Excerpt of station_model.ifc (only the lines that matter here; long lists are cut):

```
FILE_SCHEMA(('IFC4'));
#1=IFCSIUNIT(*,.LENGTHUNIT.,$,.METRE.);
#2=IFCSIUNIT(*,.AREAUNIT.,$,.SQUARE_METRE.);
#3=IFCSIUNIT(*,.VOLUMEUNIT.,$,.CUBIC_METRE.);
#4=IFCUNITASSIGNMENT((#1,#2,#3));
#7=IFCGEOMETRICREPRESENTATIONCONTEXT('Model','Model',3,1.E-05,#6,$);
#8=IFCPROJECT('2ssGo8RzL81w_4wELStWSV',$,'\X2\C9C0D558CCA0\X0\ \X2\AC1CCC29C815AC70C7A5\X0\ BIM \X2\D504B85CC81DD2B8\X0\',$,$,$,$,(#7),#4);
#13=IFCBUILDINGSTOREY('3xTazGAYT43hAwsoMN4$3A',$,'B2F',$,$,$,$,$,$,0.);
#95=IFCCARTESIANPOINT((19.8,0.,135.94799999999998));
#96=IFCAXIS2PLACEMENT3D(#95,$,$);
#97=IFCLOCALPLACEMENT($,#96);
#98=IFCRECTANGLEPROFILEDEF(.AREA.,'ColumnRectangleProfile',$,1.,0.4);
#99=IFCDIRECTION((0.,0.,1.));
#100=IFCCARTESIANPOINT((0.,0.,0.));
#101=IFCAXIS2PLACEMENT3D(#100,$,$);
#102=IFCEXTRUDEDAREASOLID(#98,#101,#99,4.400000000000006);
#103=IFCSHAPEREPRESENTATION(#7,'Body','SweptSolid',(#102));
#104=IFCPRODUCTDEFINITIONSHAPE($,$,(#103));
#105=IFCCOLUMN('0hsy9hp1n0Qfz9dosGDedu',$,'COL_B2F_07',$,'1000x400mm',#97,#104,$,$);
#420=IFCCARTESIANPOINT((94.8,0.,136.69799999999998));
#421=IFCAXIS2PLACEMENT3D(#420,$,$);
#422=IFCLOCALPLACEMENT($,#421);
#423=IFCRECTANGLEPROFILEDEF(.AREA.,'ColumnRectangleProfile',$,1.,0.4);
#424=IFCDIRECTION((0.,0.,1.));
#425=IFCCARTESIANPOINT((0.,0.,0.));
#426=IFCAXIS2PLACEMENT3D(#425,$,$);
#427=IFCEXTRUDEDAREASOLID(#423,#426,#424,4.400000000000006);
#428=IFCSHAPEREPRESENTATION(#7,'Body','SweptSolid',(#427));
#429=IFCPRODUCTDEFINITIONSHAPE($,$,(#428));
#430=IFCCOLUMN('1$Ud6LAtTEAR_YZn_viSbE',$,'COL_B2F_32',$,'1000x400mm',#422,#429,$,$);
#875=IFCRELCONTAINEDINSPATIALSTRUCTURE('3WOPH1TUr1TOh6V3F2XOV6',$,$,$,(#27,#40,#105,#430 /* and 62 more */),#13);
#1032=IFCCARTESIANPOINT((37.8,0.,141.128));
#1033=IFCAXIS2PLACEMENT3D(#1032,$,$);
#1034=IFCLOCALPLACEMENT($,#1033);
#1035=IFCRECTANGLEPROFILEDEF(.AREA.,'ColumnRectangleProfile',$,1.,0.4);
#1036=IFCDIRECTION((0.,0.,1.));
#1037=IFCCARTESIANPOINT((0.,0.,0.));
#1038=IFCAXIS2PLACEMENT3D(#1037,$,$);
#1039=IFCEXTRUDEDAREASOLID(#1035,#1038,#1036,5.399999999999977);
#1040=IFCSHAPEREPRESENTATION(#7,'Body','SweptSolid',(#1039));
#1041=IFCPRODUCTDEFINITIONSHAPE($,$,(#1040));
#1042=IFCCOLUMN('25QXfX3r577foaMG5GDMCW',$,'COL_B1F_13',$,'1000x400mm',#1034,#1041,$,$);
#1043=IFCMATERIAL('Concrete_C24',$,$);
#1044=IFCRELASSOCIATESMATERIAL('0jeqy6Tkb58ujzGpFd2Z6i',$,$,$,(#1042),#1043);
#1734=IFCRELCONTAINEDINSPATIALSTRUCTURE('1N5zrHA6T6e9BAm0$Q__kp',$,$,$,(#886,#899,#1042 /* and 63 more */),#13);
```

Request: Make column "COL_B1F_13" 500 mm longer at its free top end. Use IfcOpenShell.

```python
import ifcopenshell
import ifcopenshell.util.unit

model = ifcopenshell.open("station_model.ifc")
unit_scale = ifcopenshell.util.unit.calculate_unit_scale(model)

member = model.by_guid("25QXfX3r577foaMG5GDMCW")
change = 0.5 / unit_scale

# The extrusion runs towards the end named, so only its depth changes.
body = next(r for r in member.Representation.Representations if r.RepresentationIdentifier == "Body")
solid = body.Items[0]
old_length = solid.Depth
solid.Depth += change

print(f"length {old_length:g} -> {solid.Depth:g}")

model.write("station_model_v2.ifc")
```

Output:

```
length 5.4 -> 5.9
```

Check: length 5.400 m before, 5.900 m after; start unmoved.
